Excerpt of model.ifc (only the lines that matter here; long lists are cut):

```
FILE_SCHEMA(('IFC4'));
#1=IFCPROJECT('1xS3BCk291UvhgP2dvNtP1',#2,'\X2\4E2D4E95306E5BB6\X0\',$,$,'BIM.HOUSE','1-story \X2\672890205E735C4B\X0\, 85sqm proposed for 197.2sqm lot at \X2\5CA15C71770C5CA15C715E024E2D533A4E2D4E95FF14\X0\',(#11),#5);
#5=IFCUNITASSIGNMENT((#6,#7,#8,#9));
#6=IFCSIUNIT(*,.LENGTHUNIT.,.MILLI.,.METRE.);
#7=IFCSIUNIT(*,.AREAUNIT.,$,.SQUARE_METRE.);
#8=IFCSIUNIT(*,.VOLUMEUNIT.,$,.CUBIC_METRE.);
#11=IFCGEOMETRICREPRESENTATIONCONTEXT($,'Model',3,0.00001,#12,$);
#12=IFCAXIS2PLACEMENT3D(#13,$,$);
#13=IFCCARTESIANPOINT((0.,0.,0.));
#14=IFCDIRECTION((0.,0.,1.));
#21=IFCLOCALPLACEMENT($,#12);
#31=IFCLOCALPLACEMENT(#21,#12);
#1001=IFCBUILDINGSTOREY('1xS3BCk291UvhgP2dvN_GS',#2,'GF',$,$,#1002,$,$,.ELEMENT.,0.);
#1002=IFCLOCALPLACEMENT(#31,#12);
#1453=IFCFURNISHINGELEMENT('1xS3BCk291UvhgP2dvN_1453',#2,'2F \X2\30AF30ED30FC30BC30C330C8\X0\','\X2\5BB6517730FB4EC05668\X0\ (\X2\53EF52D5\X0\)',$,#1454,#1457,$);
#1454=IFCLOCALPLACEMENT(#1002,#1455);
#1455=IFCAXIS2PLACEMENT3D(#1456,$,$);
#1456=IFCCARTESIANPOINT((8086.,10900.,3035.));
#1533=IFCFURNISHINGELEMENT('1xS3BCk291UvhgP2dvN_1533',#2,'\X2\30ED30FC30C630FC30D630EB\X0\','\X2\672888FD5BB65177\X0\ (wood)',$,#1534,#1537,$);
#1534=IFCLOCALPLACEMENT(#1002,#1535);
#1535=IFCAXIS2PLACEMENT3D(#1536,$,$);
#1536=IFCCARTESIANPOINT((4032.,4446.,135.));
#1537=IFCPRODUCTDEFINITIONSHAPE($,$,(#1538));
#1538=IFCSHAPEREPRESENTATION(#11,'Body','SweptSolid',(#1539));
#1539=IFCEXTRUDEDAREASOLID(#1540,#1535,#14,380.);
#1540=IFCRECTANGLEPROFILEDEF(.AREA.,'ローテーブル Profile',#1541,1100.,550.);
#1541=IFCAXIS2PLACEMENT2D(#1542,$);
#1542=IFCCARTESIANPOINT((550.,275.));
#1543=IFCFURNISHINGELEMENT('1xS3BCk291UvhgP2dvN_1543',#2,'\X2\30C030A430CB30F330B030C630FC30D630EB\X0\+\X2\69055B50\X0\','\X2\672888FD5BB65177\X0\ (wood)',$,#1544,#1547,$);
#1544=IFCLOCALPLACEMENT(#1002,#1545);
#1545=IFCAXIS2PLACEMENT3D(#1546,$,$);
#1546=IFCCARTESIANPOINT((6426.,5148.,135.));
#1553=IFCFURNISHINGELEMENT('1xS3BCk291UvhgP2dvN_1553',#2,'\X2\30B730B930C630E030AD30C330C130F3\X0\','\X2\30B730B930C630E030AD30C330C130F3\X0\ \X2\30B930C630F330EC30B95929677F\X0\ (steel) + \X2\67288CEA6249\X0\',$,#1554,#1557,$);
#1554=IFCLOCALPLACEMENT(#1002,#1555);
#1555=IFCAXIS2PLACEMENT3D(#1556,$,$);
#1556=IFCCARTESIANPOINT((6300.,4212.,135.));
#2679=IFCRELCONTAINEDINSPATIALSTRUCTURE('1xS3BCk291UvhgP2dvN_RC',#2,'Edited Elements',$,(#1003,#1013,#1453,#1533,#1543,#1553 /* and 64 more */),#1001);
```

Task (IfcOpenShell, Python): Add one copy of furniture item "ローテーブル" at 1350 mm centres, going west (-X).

```python
import numpy as np
import ifcopenshell
import ifcopenshell.api.geometry
import ifcopenshell.api.root
import ifcopenshell.util.element
import ifcopenshell.util.placement
import ifcopenshell.util.unit

model = ifcopenshell.open("model.ifc")
unit_scale = ifcopenshell.util.unit.calculate_unit_scale(model)


def reuse_history(source, copy):
    """copy_class also copies each property set's owner history, people and application; keep the originals."""
    for rel in copy.IsDefinedBy:
        if rel.is_a("IfcRelDefinesByProperties") and (history := rel.RelatingPropertyDefinition.OwnerHistory):
            rel.RelatingPropertyDefinition.OwnerHistory = source.OwnerHistory
            ifcopenshell.util.element.remove_deep2(model, history)


source = model.by_id(1533)
base = ifcopenshell.util.placement.get_local_placement(source.ObjectPlacement)
step = np.array([-1.0, 0.0, 0.0]) * 1.35 / unit_scale

for i in range(1, 2):
    copy = ifcopenshell.api.root.copy_class(model, product=source)
    copy.Representation = ifcopenshell.util.element.copy_deep(
        model, source.Representation, exclude=["IfcGeometricRepresentationContext", "IfcRepresentationMap"]
    )
    reuse_history(source, copy)
    matrix = base.copy()
    matrix[:3, 3] += i * step
    print("added at", matrix[:3, 3].round(3) + 0.0)
    ifcopenshell.api.geometry.edit_object_placement(model, product=copy, matrix=matrix, is_si=False)

model.write("model_updated.ifc")
```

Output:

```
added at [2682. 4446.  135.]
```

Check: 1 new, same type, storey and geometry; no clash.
